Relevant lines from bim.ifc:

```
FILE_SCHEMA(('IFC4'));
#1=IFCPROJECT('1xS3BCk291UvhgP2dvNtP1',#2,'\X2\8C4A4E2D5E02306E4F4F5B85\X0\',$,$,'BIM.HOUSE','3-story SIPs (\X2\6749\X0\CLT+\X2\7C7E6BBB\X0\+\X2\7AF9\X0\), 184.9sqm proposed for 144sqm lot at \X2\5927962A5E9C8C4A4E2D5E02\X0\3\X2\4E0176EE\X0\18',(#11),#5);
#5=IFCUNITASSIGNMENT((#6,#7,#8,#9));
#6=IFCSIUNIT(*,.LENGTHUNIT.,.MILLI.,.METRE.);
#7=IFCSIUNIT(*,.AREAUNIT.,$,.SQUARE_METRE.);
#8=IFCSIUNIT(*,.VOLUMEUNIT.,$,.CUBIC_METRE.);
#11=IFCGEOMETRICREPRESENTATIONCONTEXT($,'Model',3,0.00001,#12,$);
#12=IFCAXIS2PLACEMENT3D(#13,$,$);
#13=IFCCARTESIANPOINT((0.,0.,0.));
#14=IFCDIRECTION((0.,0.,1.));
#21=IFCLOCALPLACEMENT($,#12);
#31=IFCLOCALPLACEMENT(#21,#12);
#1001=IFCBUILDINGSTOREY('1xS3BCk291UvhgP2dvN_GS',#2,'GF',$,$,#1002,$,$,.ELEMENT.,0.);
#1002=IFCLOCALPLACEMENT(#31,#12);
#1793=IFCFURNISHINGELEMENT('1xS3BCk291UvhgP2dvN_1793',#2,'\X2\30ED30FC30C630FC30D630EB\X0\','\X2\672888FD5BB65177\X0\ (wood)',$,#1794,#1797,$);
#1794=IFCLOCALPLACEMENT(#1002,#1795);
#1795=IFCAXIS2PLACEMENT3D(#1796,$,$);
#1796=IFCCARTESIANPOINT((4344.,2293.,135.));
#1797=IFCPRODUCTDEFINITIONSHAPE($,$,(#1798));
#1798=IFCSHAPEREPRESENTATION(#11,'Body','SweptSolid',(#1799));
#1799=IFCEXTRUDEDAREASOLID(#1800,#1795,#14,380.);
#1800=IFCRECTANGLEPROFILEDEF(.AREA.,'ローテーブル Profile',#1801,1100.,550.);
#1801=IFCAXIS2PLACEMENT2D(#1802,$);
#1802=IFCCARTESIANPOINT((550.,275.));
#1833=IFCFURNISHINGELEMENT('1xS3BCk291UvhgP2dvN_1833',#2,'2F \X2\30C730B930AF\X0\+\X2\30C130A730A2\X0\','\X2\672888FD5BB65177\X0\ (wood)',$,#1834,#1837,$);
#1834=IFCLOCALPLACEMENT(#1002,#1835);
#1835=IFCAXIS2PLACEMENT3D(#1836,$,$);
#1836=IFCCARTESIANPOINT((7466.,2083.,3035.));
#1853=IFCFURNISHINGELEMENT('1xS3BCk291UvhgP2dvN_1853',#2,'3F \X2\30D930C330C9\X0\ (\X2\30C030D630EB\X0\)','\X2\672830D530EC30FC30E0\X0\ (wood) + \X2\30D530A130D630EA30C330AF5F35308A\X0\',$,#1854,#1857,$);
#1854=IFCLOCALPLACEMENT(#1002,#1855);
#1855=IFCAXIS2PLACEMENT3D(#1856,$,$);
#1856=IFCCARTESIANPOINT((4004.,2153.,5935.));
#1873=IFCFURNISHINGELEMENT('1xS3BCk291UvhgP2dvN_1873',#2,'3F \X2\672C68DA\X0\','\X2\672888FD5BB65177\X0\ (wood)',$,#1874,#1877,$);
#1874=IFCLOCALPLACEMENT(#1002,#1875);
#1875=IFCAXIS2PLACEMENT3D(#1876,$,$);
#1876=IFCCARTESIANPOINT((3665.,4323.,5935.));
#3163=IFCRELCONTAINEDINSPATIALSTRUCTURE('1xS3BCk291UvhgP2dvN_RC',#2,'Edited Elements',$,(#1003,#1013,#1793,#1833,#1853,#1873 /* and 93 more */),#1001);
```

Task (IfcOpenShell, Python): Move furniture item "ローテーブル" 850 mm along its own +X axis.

```python
import ifcopenshell
import ifcopenshell.api.geometry
import ifcopenshell.util.placement

model = ifcopenshell.open("bim.ifc")

item = model.by_guid("1xS3BCk291UvhgP2dvN_1793")
matrix = ifcopenshell.util.placement.get_local_placement(item.ObjectPlacement)
matrix[:3, 3] += matrix[:3, 0] * 850.0
ifcopenshell.api.geometry.edit_object_placement(model, product=item, matrix=matrix, is_si=False)

print(ifcopenshell.util.placement.get_local_placement(item.ObjectPlacement).round(3) + 0.0)

model.write("bim_updated.ifc")
```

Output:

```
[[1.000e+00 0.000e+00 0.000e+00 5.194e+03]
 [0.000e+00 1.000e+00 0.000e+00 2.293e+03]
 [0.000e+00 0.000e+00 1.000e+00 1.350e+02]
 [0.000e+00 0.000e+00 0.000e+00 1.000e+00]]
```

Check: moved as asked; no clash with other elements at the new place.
